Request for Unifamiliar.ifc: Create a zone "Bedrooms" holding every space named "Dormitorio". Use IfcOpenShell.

First a look at what the model holds.

```python
import ifcopenshell

model = ifcopenshell.open("Unifamiliar.ifc")
print(model.schema)
seen = {}
for space in model.by_type("IfcSpace"):
    seen[space.LongName] = seen.get(space.LongName, 0) + 1
for name, count in sorted(seen.items(), key=str):
    print(count, "x", name)
print("zones:", [z.Name for z in model.by_type("IfcZone")][:20])
```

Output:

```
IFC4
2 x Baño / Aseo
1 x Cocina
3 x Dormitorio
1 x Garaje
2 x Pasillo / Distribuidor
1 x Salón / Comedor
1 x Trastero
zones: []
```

```python
import ifcopenshell
import ifcopenshell.api.group
import ifcopenshell.api.root

model = ifcopenshell.open("Unifamiliar.ifc")

names = {"Dormitorio"}
spaces = [s for s in model.by_type("IfcSpace") if s.LongName in names]

zone = ifcopenshell.api.root.create_entity(model, ifc_class="IfcZone", name="Bedrooms")
ifcopenshell.api.group.assign_group(model, products=spaces, group=zone)
print(len(spaces), "spaces in", zone.Name)

model.write("Unifamiliar_rev.ifc")
```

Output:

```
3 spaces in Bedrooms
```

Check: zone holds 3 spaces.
